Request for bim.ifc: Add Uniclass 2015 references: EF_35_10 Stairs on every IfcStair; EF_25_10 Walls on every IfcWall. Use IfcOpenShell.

First a look at what the model holds.

```python
import ifcopenshell

model = ifcopenshell.open("bim.ifc")
print(model.schema)
print("classifications:", [c.Name for c in model.by_type("IfcClassification")])
for ifc_class in ("IfcDoor", "IfcRoof", "IfcStair", "IfcWall", "IfcWindow"):
    print(ifc_class, len(model.by_type(ifc_class)))
```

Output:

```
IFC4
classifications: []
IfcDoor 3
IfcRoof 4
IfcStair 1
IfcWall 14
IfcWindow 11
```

```python
import ifcopenshell
import ifcopenshell.api.classification

model = ifcopenshell.open("bim.ifc")

system = ifcopenshell.api.classification.add_classification(model, classification="Uniclass 2015")

codes = {
    "IfcStair": ("EF_35_10", "Stairs"),
    "IfcWall": ("EF_25_10", "Walls"),
}
for ifc_class, (code, name) in codes.items():
    products = model.by_type(ifc_class)
    ifcopenshell.api.classification.add_reference(
        model, products=products, classification=system, identification=code, name=name
    )
    print(code, len(products))

model.write("bim_rev.ifc")
```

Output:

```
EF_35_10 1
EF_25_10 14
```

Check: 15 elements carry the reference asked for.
